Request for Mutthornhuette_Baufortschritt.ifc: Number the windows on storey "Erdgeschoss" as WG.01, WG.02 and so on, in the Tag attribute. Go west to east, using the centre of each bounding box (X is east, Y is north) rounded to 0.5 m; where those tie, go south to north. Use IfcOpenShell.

First a look at what the model holds.

```python
import ifcopenshell
import ifcopenshell.util.element
import ifcopenshell.util.placement

model = ifcopenshell.open("Mutthornhuette_Baufortschritt.ifc")
print(model.schema)
storey = next(s for s in model.by_type("IfcBuildingStorey") if s.Name == "Erdgeschoss")
windows = [e for e in ifcopenshell.util.element.get_decomposition(storey) if e.is_a("IfcWindow")]
for e in sorted(windows, key=lambda e: e.id()):
    origin = ifcopenshell.util.placement.get_local_placement(e.ObjectPlacement)[:3, 3]
    print(e.id(), e.Tag, e.Name, origin.round(2) + 0.0, sep=" | ")
```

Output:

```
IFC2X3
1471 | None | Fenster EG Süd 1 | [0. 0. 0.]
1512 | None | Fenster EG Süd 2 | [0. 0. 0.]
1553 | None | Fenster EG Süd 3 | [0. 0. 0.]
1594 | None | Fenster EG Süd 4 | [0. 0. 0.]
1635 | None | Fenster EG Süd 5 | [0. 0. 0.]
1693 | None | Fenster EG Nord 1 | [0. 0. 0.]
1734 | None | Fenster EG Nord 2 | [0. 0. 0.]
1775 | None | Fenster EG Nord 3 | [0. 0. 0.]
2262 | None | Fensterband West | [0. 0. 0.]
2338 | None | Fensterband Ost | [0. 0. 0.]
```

```python
import ifcopenshell
import ifcopenshell.geom
import ifcopenshell.util.element
import ifcopenshell.util.shape

model = ifcopenshell.open("Mutthornhuette_Baufortschritt.ifc")
settings = ifcopenshell.geom.settings()
settings.set("use-world-coords", True)


def centre(element):
    shape = ifcopenshell.geom.create_shape(settings, element)
    return ifcopenshell.util.shape.get_bbox_centroid(shape.geometry)


storey = next(s for s in model.by_type("IfcBuildingStorey") if s.Name == "Erdgeschoss")
windows = [e for e in ifcopenshell.util.element.get_decomposition(storey) if e.is_a("IfcWindow")]

# Insertion points can sit at a corner or the storey origin, so sort by the geometry (in metres).
centres = {e: centre(e) for e in windows}
windows.sort(key=lambda e: (round(centres[e][0] / 0.5), centres[e][1]))

for i, e in enumerate(windows, start=1):
    number = f"WG.{i:02d}"
    e.Tag = number
    print(e.id(), number)

model.write("Mutthornhuette_Baufortschritt-out.ifc")
```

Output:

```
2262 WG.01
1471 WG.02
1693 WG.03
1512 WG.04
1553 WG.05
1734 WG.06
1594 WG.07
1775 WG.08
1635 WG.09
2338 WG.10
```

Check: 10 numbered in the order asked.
